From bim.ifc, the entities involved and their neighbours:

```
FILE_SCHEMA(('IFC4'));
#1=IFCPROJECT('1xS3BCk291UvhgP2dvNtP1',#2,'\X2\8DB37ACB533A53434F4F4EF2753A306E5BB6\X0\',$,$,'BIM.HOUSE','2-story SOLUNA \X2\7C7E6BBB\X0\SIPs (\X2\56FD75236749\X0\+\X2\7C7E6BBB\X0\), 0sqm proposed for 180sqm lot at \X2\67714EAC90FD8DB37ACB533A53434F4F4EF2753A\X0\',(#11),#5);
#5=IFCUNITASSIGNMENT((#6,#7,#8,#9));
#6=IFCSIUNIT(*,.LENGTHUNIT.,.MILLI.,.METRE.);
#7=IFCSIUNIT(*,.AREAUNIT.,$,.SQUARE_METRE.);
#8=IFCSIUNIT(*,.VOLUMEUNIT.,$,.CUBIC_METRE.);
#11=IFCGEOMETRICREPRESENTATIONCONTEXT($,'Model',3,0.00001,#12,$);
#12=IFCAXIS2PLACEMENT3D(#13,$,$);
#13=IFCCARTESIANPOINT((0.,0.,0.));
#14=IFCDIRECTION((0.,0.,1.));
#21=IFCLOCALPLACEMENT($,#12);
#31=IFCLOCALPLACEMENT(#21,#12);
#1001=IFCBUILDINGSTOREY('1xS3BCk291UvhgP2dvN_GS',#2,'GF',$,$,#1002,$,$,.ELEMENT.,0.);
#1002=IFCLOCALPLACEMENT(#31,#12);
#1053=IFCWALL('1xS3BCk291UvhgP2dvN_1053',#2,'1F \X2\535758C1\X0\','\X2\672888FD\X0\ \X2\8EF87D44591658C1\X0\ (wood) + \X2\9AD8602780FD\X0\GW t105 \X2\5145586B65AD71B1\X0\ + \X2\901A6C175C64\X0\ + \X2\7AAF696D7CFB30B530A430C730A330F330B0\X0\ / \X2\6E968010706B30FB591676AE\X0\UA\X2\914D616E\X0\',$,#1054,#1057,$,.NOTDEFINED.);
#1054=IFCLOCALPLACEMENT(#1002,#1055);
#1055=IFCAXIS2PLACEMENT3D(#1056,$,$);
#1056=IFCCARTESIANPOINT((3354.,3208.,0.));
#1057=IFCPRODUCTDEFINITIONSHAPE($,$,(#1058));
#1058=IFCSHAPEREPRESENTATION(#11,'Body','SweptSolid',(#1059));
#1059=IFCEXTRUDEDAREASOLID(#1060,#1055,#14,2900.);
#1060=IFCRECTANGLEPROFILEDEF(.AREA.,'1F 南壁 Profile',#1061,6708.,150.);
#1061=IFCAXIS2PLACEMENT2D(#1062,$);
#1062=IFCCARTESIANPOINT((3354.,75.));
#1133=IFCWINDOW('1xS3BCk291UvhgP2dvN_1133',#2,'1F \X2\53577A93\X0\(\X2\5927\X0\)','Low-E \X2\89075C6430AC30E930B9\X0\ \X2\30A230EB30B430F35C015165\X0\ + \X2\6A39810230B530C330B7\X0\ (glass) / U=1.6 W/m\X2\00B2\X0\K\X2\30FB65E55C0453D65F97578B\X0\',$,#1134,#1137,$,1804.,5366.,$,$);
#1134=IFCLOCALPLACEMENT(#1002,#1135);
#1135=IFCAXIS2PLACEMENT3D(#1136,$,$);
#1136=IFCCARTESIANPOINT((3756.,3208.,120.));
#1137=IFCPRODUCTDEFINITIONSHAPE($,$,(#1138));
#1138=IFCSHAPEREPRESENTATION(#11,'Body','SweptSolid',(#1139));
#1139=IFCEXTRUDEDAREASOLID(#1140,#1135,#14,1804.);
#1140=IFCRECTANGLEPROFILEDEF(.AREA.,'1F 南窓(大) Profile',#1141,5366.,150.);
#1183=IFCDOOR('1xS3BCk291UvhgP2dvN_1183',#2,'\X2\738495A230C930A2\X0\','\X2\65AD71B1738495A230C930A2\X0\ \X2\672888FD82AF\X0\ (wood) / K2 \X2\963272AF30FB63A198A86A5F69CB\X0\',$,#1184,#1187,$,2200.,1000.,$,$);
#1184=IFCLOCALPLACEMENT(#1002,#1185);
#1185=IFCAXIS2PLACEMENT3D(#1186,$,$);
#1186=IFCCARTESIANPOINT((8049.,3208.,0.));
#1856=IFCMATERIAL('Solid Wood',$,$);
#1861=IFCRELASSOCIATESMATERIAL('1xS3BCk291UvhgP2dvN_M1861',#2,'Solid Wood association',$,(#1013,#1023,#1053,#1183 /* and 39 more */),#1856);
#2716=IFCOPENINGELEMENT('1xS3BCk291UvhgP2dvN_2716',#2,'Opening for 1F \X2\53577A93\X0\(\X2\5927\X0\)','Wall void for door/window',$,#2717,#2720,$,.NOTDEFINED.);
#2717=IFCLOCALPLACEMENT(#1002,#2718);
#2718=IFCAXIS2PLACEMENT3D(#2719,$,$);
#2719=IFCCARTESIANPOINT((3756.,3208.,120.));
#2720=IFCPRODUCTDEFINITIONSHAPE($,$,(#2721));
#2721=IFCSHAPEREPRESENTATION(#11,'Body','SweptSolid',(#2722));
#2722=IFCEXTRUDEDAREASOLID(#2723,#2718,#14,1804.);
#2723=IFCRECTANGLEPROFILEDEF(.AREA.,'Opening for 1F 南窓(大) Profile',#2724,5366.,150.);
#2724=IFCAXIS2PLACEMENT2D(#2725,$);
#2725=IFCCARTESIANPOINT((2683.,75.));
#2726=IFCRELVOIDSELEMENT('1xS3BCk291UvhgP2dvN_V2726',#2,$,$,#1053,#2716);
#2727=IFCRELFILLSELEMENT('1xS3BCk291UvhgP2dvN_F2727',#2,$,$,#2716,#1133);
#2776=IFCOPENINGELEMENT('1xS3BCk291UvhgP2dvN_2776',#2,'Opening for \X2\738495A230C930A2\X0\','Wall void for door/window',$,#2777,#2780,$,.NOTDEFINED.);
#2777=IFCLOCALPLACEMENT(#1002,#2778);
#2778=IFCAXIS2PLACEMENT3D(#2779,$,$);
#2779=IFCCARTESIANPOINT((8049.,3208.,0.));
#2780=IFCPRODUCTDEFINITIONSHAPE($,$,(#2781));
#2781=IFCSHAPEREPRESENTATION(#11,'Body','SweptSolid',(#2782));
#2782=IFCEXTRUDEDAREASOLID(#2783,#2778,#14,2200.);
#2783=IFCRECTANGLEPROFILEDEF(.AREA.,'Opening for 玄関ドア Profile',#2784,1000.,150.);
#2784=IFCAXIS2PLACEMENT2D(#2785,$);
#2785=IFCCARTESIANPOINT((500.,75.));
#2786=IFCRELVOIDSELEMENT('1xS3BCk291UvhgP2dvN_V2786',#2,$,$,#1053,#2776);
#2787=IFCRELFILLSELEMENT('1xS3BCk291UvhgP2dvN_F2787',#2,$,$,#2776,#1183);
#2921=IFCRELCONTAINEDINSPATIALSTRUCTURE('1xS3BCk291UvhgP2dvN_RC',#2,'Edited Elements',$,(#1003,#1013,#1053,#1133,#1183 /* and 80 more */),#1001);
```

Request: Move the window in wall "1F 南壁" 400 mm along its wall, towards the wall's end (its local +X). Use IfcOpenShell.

```python
import ifcopenshell
import ifcopenshell.api.geometry
import ifcopenshell.util.placement

model = ifcopenshell.open("bim.ifc")

window = model.by_guid("1xS3BCk291UvhgP2dvN_1133")
opening = window.FillsVoids[0].RelatingOpeningElement
wall = opening.VoidsElements[0].RelatingBuildingElement

wall_matrix = ifcopenshell.util.placement.get_local_placement(wall.ObjectPlacement)
shift = wall_matrix[:3, 0] * 400.0
before = ifcopenshell.util.placement.get_local_placement(window.ObjectPlacement)[:3, 3].copy()

# The window is not placed relative to its opening, so move both.
for product in (opening, window):
    matrix = ifcopenshell.util.placement.get_local_placement(product.ObjectPlacement)
    matrix[:3, 3] += shift
    ifcopenshell.api.geometry.edit_object_placement(model, product=product, matrix=matrix, is_si=False)

after = ifcopenshell.util.placement.get_local_placement(window.ObjectPlacement)[:3, 3]
print("window moved by", (after - before).round(3) + 0.0)

model.write("bim_updated.ifc")
```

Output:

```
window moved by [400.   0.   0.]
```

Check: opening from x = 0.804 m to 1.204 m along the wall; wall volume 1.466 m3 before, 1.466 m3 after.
